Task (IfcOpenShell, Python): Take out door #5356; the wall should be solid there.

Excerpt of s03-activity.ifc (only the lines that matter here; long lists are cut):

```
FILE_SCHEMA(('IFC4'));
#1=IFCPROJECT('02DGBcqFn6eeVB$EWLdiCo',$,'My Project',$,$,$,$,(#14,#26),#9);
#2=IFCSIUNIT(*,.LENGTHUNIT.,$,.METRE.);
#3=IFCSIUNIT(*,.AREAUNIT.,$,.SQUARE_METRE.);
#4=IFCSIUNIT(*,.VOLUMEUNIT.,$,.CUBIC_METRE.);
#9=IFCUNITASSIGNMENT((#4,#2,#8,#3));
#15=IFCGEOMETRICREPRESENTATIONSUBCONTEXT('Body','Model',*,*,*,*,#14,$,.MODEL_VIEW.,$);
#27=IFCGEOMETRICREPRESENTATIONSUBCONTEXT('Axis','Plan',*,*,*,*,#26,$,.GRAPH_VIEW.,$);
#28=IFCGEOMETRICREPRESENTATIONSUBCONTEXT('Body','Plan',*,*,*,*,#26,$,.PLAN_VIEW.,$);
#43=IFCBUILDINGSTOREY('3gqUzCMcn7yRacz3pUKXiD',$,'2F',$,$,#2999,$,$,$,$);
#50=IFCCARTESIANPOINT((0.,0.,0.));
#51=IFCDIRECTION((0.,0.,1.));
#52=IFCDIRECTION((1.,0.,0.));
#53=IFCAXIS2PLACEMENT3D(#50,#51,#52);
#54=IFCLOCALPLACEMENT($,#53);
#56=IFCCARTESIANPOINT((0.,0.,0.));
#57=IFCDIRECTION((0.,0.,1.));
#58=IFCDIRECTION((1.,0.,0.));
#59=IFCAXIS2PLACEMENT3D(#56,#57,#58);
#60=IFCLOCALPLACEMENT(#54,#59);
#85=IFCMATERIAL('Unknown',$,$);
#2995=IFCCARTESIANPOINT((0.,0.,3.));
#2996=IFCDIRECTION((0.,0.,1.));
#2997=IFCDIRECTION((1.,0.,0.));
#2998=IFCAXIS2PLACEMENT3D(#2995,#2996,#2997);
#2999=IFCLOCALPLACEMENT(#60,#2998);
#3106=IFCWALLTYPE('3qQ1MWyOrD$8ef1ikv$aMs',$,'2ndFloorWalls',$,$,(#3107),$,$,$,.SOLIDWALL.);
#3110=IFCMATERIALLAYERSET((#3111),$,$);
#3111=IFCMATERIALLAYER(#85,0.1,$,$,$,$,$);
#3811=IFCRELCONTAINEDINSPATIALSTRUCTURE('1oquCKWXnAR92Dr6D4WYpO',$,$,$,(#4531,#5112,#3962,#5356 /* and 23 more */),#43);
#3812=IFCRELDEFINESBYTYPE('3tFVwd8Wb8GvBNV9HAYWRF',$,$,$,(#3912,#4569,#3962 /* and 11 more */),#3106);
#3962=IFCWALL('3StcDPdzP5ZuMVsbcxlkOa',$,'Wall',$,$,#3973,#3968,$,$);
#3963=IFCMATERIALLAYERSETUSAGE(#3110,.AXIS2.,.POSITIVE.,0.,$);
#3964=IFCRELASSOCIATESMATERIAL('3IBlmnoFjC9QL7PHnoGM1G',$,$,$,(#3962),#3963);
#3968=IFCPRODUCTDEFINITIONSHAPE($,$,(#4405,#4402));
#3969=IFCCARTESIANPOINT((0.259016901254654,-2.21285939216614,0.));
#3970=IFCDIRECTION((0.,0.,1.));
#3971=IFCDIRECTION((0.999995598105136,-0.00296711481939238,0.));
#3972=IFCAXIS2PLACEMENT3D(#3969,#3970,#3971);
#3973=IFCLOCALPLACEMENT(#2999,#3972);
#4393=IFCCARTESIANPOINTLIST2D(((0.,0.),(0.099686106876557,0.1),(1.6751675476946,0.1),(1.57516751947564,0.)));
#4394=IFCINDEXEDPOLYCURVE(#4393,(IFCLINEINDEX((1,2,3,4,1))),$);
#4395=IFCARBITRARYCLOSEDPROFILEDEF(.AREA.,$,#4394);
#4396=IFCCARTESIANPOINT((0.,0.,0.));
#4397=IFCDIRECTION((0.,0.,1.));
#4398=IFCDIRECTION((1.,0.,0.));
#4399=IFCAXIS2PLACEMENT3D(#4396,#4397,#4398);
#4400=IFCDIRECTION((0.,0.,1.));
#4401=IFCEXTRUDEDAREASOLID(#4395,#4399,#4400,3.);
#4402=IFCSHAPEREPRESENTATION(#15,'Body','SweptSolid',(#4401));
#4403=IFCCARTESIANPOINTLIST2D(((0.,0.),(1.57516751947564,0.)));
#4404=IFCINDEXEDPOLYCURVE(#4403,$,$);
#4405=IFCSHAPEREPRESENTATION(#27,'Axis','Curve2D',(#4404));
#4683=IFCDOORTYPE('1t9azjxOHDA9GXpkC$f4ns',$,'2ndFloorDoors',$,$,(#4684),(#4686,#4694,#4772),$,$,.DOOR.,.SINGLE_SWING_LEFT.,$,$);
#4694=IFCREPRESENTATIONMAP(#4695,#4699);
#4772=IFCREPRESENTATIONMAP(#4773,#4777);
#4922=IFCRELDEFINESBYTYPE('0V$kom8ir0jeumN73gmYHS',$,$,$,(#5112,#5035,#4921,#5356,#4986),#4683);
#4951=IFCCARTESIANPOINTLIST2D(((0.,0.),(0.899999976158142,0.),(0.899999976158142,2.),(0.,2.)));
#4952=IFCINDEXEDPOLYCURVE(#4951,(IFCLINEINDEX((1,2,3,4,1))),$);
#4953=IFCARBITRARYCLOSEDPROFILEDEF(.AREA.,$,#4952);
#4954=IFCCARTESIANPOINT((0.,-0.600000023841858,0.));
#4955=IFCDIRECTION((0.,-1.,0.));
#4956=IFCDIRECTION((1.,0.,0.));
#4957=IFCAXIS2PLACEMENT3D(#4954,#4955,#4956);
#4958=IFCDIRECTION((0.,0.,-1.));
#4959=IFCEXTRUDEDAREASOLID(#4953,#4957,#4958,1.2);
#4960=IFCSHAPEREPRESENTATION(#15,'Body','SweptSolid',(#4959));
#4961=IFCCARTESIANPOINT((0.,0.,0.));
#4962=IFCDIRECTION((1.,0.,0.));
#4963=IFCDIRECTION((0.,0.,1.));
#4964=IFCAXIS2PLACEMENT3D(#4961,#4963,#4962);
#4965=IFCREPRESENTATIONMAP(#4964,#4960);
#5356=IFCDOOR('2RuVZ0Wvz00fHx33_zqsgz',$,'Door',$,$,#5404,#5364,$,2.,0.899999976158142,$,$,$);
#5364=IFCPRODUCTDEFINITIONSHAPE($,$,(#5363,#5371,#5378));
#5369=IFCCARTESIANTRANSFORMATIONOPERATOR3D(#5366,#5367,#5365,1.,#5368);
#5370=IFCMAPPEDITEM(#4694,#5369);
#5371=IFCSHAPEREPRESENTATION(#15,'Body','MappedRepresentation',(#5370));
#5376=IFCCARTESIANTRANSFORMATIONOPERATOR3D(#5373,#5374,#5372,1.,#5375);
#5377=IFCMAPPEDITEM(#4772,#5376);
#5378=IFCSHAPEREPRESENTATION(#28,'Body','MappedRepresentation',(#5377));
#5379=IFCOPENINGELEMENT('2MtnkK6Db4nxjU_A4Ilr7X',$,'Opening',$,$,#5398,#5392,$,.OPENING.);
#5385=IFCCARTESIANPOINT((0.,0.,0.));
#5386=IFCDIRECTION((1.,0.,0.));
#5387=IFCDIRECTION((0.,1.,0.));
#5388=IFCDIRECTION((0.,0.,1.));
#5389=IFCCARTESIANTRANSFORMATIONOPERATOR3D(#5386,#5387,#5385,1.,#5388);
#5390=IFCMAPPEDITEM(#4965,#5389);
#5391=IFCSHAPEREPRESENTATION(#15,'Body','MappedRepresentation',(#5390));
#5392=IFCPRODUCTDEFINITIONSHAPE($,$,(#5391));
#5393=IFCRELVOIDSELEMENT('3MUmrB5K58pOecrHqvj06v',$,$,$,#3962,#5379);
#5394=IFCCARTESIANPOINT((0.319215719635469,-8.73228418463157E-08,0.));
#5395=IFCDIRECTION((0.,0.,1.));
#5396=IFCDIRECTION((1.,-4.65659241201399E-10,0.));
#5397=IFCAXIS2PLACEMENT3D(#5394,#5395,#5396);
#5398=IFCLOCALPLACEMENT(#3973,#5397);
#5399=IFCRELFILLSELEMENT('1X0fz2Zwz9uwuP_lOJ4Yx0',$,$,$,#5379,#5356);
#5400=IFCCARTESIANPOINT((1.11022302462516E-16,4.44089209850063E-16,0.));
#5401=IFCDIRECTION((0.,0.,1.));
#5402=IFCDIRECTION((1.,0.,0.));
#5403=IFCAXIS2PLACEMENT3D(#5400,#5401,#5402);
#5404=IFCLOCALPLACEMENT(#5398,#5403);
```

```python
import ifcopenshell
import ifcopenshell.api.feature
import ifcopenshell.api.root
import ifcopenshell.geom
import ifcopenshell.util.shape

model = ifcopenshell.open("s03-activity.ifc")
settings = ifcopenshell.geom.settings()


def volume(element):
    """Net volume in cubic metres, openings subtracted."""
    shape = ifcopenshell.geom.create_shape(settings, element)
    return ifcopenshell.util.shape.get_volume(shape.geometry)


door = model.by_guid("2RuVZ0Wvz00fHx33_zqsgz")
opening = door.FillsVoids[0].RelatingOpeningElement
wall = opening.VoidsElements[0].RelatingBuildingElement
before = volume(wall)

ifcopenshell.api.root.remove_product(model, product=door)
ifcopenshell.api.feature.remove_feature(model, feature=opening)

after = volume(wall)

print(f"wall volume {before:.3f} -> {after:.3f} m3")

model.write("s03-activity_updated.ifc")
```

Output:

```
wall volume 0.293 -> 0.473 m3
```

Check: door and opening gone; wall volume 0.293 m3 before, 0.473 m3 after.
